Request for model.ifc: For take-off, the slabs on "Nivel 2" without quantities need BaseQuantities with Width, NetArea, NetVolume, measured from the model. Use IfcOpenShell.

First a look at what the model holds.

```python
import ifcopenshell
import ifcopenshell.util.element
import ifcopenshell.util.unit

model = ifcopenshell.open("model.ifc")
print(model.schema)
for unit_type in ("LENGTHUNIT", "AREAUNIT", "VOLUMEUNIT"):
    print(unit_type, ifcopenshell.util.unit.calculate_unit_scale(model, unit_type))
storey = next(s for s in model.by_type("IfcBuildingStorey") if s.Name == "Nivel 2")
slabs = [e for e in ifcopenshell.util.element.get_decomposition(storey) if e.is_a("IfcSlab")]
for e in sorted(slabs, key=lambda e: e.id()):
    print(e.id(), e.is_a(), e.Name, list(ifcopenshell.util.element.get_psets(e, qtos_only=True)), sep=" | ")
```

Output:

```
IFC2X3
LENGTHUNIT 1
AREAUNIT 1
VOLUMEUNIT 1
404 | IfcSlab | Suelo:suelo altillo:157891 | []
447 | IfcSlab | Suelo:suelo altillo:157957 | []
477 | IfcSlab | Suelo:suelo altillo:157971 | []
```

```python
import ifcopenshell
import ifcopenshell.api.pset
import ifcopenshell.geom
import ifcopenshell.util.element
import ifcopenshell.util.shape
import ifcopenshell.util.unit

model = ifcopenshell.open("model.ifc")
unit_scale = ifcopenshell.util.unit.calculate_unit_scale(model)
area_scale = ifcopenshell.util.unit.calculate_unit_scale(model, "AREAUNIT")
volume_scale = ifcopenshell.util.unit.calculate_unit_scale(model, "VOLUMEUNIT")
settings = ifcopenshell.geom.settings()

storey = next(s for s in model.by_type("IfcBuildingStorey") if s.Name == "Nivel 2")
slabs = [e for e in ifcopenshell.util.element.get_decomposition(storey) if e.is_a("IfcSlab")]

for e in sorted(slabs, key=lambda e: e.id()):
    if ifcopenshell.util.element.get_psets(e, qtos_only=True, should_inherit=False):
        continue
    # Geometry comes back in metres, in the element's own axes.
    shape = ifcopenshell.geom.create_shape(settings, e)
    values = {
        "Width": ifcopenshell.util.shape.get_z(shape.geometry) / unit_scale,
        "NetArea": ifcopenshell.util.shape.get_footprint_area(shape.geometry) / area_scale,
        "NetVolume": ifcopenshell.util.shape.get_volume(shape.geometry) / volume_scale,
    }
    qto = ifcopenshell.api.pset.add_qto(model, product=e, name="BaseQuantities")
    ifcopenshell.api.pset.edit_qto(model, qto=qto, properties=values)
    print(e.id(), {k: round(v, 3) for k, v in values.items()})

model.write("model_rev.ifc")
```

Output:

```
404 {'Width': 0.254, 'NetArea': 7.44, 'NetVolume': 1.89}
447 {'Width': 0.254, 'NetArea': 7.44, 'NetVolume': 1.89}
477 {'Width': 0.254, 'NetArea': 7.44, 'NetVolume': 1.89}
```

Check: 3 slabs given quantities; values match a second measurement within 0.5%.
